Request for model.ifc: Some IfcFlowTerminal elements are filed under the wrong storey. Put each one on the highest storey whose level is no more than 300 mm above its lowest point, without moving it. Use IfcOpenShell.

First a look at what the model holds.

```python
import ifcopenshell
import ifcopenshell.util.element
import ifcopenshell.util.placement

model = ifcopenshell.open("model.ifc")
print(model.schema)
for storey in model.by_type("IfcBuildingStorey"):
    level = ifcopenshell.util.placement.get_storey_elevation(storey)
    count = sum(e.is_a("IfcFlowTerminal") for e in ifcopenshell.util.element.get_contained(storey))
    print(storey.id(), storey.Name, round(level, 3), count, sep=" | ")
```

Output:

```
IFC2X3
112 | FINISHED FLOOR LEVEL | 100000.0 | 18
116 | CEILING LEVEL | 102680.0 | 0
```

```python
import ifcopenshell
import ifcopenshell.api.spatial
import ifcopenshell.geom
import ifcopenshell.util.element
import ifcopenshell.util.placement
import ifcopenshell.util.shape
import ifcopenshell.util.unit

model = ifcopenshell.open("model.ifc")
unit_scale = ifcopenshell.util.unit.calculate_unit_scale(model)
settings = ifcopenshell.geom.settings()

levels = sorted(
    ((ifcopenshell.util.placement.get_storey_elevation(s) * unit_scale, s) for s in model.by_type("IfcBuildingStorey")),
    key=lambda pair: pair[0],
)

for e in model.by_type("IfcFlowTerminal"):
    current = e.ContainedInStructure[0].RelatingStructure if e.ContainedInStructure else None
    if current is None or not current.is_a("IfcBuildingStorey"):
        continue
    shape = ifcopenshell.geom.create_shape(settings, e)
    bottom = ifcopenshell.util.shape.get_shape_bottom_elevation(shape, shape.geometry)
    below = [s for level, s in levels if level <= bottom + 0.3]
    storey = below[-1] if below else levels[0][1]
    if storey != current:
        # assign_container keeps the world position.
        ifcopenshell.api.spatial.assign_container(model, products=[e], relating_structure=storey)
        print(e.id(), current.Name, "->", storey.Name)

model.write("model_v2.ifc")
```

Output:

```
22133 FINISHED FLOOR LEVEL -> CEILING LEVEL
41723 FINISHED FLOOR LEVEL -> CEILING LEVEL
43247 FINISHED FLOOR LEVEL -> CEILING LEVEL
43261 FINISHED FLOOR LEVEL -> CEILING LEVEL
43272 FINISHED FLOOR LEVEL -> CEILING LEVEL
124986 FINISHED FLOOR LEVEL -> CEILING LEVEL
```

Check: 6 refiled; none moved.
